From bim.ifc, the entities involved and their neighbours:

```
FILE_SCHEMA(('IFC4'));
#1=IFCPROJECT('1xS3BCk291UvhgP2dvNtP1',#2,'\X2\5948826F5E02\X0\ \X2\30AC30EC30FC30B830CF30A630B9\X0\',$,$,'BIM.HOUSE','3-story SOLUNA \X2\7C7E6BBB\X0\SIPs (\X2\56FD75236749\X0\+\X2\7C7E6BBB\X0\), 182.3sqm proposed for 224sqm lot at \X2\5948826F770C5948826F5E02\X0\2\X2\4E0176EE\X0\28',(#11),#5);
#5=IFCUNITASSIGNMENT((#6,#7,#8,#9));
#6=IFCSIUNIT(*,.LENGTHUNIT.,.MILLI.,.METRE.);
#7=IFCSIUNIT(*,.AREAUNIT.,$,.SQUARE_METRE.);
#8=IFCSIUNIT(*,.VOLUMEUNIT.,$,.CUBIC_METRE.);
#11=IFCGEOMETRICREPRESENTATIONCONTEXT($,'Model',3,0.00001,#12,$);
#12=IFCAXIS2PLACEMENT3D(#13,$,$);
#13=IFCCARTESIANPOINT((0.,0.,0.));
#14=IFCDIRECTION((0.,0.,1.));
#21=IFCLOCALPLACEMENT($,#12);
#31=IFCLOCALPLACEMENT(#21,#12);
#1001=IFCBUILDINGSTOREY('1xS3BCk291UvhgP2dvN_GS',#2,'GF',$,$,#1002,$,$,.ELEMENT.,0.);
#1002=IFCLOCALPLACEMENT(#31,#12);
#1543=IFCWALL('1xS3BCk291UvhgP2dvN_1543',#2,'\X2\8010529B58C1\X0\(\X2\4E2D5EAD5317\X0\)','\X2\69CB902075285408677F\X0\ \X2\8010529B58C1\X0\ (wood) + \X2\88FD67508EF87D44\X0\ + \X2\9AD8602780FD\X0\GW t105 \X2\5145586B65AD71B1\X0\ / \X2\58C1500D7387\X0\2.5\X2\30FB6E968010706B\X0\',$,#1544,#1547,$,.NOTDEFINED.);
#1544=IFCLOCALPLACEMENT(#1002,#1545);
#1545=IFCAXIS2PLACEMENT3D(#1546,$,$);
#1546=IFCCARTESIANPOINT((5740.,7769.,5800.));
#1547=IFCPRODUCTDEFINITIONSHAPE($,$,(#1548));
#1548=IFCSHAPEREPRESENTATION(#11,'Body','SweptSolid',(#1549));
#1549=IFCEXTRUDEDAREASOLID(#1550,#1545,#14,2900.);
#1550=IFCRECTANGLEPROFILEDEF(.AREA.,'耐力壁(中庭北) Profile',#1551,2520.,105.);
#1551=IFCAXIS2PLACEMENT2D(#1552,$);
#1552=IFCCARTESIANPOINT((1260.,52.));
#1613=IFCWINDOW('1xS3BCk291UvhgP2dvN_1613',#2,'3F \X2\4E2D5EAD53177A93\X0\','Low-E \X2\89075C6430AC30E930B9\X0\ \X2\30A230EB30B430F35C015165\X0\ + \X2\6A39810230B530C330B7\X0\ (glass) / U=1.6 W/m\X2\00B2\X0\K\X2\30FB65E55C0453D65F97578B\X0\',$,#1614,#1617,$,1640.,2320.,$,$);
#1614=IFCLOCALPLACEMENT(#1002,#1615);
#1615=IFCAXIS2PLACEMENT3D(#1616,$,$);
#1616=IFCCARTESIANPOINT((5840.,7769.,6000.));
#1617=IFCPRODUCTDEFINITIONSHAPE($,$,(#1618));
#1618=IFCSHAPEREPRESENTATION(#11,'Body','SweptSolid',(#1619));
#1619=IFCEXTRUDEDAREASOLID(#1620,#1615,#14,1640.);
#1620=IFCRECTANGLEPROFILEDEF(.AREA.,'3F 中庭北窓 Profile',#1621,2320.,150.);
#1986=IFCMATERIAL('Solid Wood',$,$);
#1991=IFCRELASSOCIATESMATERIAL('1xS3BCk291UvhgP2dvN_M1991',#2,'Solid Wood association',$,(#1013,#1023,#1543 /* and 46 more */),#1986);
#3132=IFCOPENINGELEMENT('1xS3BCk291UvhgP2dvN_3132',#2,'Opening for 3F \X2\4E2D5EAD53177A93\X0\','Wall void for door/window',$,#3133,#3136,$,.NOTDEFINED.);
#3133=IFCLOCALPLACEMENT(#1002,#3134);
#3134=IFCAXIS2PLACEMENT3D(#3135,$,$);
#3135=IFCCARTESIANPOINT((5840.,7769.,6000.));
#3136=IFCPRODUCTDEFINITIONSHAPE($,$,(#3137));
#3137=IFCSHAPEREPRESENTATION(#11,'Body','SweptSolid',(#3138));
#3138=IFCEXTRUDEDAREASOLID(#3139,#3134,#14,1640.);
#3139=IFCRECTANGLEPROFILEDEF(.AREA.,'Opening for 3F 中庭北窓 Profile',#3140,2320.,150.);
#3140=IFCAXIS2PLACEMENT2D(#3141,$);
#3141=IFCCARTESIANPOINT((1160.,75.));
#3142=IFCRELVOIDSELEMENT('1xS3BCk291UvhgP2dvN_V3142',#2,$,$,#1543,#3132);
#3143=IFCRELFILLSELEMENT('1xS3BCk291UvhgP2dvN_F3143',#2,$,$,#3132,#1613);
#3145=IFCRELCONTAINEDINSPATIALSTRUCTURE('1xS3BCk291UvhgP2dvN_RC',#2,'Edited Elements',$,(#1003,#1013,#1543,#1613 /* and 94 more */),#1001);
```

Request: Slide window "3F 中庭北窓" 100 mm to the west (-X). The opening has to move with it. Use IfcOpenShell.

```python
import ifcopenshell
import ifcopenshell.api.geometry
import ifcopenshell.util.placement

model = ifcopenshell.open("bim.ifc")

window = model.by_id(1613)
opening = window.FillsVoids[0].RelatingOpeningElement
wall = opening.VoidsElements[0].RelatingBuildingElement

wall_matrix = ifcopenshell.util.placement.get_local_placement(wall.ObjectPlacement)
shift = wall_matrix[:3, 0] * -100.0
before = ifcopenshell.util.placement.get_local_placement(window.ObjectPlacement)[:3, 3].copy()

# The window is not placed relative to its opening, so move both.
for product in (opening, window):
    matrix = ifcopenshell.util.placement.get_local_placement(product.ObjectPlacement)
    matrix[:3, 3] += shift
    ifcopenshell.api.geometry.edit_object_placement(model, product=product, matrix=matrix, is_si=False)

after = ifcopenshell.util.placement.get_local_placement(window.ObjectPlacement)[:3, 3]
print("window moved by", (after - before).round(3) + 0.0)

model.write("bim-out.ifc")
```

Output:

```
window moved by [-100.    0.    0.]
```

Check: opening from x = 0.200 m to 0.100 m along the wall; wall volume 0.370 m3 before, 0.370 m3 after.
